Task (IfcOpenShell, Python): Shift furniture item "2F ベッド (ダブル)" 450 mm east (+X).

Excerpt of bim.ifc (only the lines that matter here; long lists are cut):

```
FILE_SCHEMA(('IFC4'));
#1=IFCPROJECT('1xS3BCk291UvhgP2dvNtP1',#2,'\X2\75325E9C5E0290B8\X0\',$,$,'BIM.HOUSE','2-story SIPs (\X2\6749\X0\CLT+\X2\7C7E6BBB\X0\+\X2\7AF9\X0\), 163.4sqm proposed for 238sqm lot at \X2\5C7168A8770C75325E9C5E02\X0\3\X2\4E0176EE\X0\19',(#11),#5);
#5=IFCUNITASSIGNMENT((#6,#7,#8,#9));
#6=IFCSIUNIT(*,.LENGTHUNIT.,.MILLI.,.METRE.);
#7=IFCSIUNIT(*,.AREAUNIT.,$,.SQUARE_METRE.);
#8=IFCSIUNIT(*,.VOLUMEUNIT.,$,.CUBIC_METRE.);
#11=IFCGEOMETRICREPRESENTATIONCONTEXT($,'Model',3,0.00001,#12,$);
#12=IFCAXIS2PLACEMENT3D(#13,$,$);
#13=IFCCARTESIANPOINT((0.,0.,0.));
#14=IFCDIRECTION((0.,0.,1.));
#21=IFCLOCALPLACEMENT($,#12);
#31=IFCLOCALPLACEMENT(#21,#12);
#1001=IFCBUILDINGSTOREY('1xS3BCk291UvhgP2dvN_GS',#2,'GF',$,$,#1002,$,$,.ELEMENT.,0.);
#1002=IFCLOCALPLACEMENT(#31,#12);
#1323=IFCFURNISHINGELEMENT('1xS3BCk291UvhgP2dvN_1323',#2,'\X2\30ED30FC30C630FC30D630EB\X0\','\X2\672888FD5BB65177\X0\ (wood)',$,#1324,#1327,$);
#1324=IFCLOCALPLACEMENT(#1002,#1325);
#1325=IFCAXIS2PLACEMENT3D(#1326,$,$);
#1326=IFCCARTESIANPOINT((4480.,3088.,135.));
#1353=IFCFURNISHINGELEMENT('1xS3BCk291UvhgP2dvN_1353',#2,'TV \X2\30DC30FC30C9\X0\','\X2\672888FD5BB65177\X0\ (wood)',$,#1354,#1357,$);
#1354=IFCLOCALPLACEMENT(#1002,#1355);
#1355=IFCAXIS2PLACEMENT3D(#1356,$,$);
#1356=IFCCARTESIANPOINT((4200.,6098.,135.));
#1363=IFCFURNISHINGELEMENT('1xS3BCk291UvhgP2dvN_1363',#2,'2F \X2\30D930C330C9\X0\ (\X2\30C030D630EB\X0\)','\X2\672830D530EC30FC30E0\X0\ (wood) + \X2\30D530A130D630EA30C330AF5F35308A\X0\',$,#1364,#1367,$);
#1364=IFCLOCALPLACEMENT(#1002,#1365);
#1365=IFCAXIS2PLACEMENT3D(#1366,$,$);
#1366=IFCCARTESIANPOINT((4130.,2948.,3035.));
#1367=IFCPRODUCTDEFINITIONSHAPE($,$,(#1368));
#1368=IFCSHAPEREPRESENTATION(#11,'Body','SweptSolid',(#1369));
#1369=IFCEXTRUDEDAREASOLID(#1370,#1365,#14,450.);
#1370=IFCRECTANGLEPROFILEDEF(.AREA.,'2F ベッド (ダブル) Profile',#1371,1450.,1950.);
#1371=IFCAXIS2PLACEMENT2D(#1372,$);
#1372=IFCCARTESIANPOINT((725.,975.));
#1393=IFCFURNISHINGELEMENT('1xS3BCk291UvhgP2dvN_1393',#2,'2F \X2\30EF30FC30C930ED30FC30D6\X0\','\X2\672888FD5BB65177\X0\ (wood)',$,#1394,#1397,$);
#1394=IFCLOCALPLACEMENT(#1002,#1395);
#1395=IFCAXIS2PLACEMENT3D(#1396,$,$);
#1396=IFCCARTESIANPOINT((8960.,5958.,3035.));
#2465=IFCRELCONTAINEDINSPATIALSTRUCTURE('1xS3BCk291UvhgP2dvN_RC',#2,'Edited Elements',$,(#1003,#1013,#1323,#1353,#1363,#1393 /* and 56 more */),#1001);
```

```python
import ifcopenshell
import ifcopenshell.api.geometry
import ifcopenshell.util.placement
import ifcopenshell.util.unit

model = ifcopenshell.open("bim.ifc")
unit_scale = ifcopenshell.util.unit.calculate_unit_scale(model)

item = model.by_guid("1xS3BCk291UvhgP2dvN_1363")
matrix = ifcopenshell.util.placement.get_local_placement(item.ObjectPlacement)
matrix[0, 3] += 0.45 / unit_scale
ifcopenshell.api.geometry.edit_object_placement(model, product=item, matrix=matrix, is_si=False)

print(ifcopenshell.util.placement.get_local_placement(item.ObjectPlacement).round(3) + 0.0)

model.write("bim_updated.ifc")
```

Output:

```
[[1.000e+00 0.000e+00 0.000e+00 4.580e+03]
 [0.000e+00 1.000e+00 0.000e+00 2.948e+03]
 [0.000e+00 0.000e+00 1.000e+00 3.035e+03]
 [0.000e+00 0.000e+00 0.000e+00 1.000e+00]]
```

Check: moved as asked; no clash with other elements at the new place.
